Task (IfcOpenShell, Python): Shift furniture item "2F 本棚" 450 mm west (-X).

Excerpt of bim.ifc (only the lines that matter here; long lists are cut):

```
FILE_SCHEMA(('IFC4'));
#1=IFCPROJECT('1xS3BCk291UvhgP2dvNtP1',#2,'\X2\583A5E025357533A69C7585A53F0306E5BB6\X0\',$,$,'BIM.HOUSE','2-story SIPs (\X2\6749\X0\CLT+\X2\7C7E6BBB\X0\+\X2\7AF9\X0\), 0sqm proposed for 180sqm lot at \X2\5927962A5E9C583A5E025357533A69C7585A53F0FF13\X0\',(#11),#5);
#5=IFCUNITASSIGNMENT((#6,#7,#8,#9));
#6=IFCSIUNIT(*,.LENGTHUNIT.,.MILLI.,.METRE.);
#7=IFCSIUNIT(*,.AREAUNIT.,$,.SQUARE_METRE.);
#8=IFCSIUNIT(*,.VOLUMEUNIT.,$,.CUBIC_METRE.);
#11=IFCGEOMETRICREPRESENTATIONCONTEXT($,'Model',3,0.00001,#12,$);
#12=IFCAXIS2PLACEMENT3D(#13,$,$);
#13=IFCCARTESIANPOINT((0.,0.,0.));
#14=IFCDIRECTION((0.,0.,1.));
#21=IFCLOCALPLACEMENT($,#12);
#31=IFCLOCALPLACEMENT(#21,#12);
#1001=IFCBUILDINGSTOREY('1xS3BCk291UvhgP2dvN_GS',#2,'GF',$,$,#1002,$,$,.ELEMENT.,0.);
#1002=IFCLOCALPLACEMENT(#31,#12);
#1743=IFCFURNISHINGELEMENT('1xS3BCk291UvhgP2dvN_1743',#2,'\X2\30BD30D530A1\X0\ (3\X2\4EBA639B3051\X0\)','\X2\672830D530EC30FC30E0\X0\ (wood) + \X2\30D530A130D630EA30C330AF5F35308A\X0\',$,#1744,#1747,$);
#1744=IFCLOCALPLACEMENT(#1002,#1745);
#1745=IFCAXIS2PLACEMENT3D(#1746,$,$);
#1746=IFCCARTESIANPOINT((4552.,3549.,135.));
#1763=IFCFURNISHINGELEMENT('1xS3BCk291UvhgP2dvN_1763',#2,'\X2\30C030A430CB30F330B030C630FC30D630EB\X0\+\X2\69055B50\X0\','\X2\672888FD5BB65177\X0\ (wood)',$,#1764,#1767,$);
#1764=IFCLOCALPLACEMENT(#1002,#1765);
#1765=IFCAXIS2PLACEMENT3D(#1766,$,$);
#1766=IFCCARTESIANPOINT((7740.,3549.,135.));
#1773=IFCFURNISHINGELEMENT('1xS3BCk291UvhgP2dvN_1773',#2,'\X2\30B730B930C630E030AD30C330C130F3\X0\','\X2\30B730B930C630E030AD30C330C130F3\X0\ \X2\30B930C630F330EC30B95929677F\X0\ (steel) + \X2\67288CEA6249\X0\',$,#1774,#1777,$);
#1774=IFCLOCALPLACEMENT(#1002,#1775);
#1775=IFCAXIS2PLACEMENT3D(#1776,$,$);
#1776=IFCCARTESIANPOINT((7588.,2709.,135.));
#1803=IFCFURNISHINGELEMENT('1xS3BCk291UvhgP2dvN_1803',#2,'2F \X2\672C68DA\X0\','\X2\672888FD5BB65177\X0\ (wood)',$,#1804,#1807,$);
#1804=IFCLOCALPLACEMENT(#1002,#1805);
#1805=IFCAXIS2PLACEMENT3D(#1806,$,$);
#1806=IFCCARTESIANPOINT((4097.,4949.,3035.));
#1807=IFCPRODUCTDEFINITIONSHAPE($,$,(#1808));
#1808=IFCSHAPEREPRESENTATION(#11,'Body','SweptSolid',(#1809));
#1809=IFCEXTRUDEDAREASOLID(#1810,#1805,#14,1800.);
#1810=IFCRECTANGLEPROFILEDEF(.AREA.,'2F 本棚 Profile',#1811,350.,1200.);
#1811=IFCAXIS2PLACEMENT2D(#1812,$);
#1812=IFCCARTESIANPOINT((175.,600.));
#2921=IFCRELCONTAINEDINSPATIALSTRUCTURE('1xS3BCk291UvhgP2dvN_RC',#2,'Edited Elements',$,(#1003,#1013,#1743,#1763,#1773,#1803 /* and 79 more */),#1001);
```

```python
import ifcopenshell
import ifcopenshell.api.geometry
import ifcopenshell.util.placement

model = ifcopenshell.open("bim.ifc")

item = model.by_guid("1xS3BCk291UvhgP2dvN_1803")
matrix = ifcopenshell.util.placement.get_local_placement(item.ObjectPlacement)
matrix[0, 3] -= 450.0
ifcopenshell.api.geometry.edit_object_placement(model, product=item, matrix=matrix, is_si=False)

print(ifcopenshell.util.placement.get_local_placement(item.ObjectPlacement).round(3) + 0.0)

model.write("bim_v2.ifc")
```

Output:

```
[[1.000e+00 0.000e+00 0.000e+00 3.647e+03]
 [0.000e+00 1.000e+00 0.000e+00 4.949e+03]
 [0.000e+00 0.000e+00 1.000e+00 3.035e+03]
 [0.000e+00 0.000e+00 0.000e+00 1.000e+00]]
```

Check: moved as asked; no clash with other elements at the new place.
